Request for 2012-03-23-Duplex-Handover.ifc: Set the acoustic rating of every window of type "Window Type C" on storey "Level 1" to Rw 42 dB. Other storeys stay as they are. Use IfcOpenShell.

First a look at what the model holds.

```python
import ifcopenshell
import ifcopenshell.util.element

model = ifcopenshell.open("2012-03-23-Duplex-Handover.ifc")
print(model.schema)
storey = next(s for s in model.by_type("IfcBuildingStorey") if s.Name == "Level 1")
windows = [e for e in ifcopenshell.util.element.get_decomposition(storey) if e.is_a("IfcWindow")]
seen = {}
for e in windows:
    element_type = ifcopenshell.util.element.get_type(e)
    key = (element_type.Name if element_type != e and element_type else None, ifcopenshell.util.element.get_pset(e, "Pset_WindowCommon", "AcousticRating"))
    seen[key] = seen.get(key, 0) + 1
for (name, value), count in sorted(seen.items(), key=str):
    print(count, "x", name, "|", value)
```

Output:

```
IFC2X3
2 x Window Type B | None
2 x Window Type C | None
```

```python
import ifcopenshell
import ifcopenshell.api.pset
import ifcopenshell.util.element

model = ifcopenshell.open("2012-03-23-Duplex-Handover.ifc")

storey = next(s for s in model.by_type("IfcBuildingStorey") if s.Name == "Level 1")
windows = [e for e in ifcopenshell.util.element.get_decomposition(storey) if e.is_a("IfcWindow")]

count = 0
for e in windows:
    element_type = ifcopenshell.util.element.get_type(e)
    if element_type in (None, e) or element_type.Name != "Window Type C":
        continue
    # add_pset returns the element's existing set when there is one.
    pset = ifcopenshell.api.pset.add_pset(model, product=e, name="Pset_WindowCommon")
    ifcopenshell.api.pset.edit_pset(model, pset=pset, properties={"AcousticRating": "Rw 42 dB"})
    count += 1

print(count, "windows updated")

model.write("2012-03-23-Duplex-Handover-out.ifc")
```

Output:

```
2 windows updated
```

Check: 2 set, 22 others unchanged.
